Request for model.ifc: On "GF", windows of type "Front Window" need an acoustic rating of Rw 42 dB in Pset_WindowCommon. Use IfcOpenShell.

First a look at what the model holds.

```python
import ifcopenshell
import ifcopenshell.util.element

model = ifcopenshell.open("model.ifc")
print(model.schema)
storey = next(s for s in model.by_type("IfcBuildingStorey") if s.Name == "GF")
windows = [e for e in ifcopenshell.util.element.get_decomposition(storey) if e.is_a("IfcWindow")]
seen = {}
for e in windows:
    element_type = ifcopenshell.util.element.get_type(e)
    key = (element_type.Name if element_type != e and element_type else None, ifcopenshell.util.element.get_pset(e, "Pset_WindowCommon", "AcousticRating"))
    seen[key] = seen.get(key, 0) + 1
for (name, value), count in sorted(seen.items(), key=str):
    print(count, "x", name, "|", value)
```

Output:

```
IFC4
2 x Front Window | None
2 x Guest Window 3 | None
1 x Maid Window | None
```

```python
import ifcopenshell
import ifcopenshell.api.pset
import ifcopenshell.util.element

model = ifcopenshell.open("model.ifc")

storey = next(s for s in model.by_type("IfcBuildingStorey") if s.Name == "GF")
windows = [e for e in ifcopenshell.util.element.get_decomposition(storey) if e.is_a("IfcWindow")]

count = 0
for e in windows:
    element_type = ifcopenshell.util.element.get_type(e)
    if element_type in (None, e) or element_type.Name != "Front Window":
        continue
    # add_pset returns the element's existing set when there is one.
    pset = ifcopenshell.api.pset.add_pset(model, product=e, name="Pset_WindowCommon")
    ifcopenshell.api.pset.edit_pset(model, pset=pset, properties={"AcousticRating": "Rw 42 dB"})
    count += 1

print(count, "windows updated")

model.write("model_rev.ifc")
```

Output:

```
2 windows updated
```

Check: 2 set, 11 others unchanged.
